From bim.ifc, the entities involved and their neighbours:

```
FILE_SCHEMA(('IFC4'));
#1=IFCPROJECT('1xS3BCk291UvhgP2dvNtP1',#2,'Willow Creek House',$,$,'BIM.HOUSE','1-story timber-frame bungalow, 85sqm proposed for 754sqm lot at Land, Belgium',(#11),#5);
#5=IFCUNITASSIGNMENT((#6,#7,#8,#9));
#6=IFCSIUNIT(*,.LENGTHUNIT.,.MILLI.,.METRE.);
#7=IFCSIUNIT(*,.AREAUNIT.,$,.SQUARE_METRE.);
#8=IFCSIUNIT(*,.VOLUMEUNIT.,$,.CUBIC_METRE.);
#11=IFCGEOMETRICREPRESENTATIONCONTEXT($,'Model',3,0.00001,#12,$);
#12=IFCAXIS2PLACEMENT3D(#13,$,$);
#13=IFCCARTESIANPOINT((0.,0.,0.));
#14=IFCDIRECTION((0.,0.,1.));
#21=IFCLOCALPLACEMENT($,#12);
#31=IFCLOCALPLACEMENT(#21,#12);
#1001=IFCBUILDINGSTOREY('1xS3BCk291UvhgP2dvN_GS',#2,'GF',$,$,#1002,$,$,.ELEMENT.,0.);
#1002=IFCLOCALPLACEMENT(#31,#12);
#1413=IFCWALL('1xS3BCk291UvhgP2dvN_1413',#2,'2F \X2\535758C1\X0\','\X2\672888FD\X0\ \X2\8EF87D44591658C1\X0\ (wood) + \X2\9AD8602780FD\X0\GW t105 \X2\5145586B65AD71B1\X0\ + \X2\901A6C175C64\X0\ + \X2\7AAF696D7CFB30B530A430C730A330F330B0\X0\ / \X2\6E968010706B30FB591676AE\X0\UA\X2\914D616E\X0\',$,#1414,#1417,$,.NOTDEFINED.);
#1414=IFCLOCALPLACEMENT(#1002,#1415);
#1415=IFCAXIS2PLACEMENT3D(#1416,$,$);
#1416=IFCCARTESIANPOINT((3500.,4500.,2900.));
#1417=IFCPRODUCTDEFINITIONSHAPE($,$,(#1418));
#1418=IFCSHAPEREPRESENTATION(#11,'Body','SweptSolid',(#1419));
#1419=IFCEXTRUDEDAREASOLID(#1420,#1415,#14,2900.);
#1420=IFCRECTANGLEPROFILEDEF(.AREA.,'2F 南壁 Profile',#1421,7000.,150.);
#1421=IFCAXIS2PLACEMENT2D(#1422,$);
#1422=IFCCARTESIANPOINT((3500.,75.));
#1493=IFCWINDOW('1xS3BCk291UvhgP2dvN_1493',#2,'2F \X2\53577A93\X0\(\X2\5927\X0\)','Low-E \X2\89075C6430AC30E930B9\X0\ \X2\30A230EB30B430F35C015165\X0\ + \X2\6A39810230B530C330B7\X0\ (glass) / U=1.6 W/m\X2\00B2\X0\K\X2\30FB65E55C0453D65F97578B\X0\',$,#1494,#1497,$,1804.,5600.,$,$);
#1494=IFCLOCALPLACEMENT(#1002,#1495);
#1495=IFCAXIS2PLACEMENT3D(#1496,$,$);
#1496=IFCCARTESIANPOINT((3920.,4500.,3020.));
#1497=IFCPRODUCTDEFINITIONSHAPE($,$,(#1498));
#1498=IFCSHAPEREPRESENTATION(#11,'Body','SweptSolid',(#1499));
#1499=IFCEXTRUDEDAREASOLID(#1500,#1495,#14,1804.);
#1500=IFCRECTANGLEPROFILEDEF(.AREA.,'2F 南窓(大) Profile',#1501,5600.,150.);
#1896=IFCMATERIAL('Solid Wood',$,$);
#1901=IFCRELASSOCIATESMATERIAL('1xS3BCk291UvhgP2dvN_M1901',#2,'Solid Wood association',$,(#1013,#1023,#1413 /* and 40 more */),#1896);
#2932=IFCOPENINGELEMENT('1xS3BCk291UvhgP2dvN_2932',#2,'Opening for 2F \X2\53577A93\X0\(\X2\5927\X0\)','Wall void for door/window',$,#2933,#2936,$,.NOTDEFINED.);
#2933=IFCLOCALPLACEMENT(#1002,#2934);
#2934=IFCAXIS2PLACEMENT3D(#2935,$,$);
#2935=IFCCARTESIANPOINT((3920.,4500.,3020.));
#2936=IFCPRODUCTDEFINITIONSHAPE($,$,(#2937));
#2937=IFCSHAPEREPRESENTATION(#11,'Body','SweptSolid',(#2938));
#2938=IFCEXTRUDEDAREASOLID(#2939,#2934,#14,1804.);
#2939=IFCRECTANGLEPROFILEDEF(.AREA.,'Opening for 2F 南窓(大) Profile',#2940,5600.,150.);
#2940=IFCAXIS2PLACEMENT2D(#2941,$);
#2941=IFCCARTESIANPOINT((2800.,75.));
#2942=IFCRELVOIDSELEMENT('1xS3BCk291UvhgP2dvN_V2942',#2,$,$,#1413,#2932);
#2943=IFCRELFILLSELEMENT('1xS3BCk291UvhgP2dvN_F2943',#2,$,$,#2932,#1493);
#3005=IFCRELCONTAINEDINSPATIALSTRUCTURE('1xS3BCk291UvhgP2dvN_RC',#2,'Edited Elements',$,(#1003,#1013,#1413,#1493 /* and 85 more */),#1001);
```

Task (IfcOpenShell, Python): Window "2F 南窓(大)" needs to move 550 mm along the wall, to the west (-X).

```python
import ifcopenshell
import ifcopenshell.api.geometry
import ifcopenshell.util.placement

model = ifcopenshell.open("bim.ifc")

window = model.by_guid("1xS3BCk291UvhgP2dvN_1493")
opening = window.FillsVoids[0].RelatingOpeningElement
wall = opening.VoidsElements[0].RelatingBuildingElement

wall_matrix = ifcopenshell.util.placement.get_local_placement(wall.ObjectPlacement)
shift = wall_matrix[:3, 0] * -550.0
before = ifcopenshell.util.placement.get_local_placement(window.ObjectPlacement)[:3, 3].copy()

# The window is not placed relative to its opening, so move both.
for product in (opening, window):
    matrix = ifcopenshell.util.placement.get_local_placement(product.ObjectPlacement)
    matrix[:3, 3] += shift
    ifcopenshell.api.geometry.edit_object_placement(model, product=product, matrix=matrix, is_si=False)

after = ifcopenshell.util.placement.get_local_placement(window.ObjectPlacement)[:3, 3]
print("window moved by", (after - before).round(3) + 0.0)

model.write("bim_rev.ifc")
```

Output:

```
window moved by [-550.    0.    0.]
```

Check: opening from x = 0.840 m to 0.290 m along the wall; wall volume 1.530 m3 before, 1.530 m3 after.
